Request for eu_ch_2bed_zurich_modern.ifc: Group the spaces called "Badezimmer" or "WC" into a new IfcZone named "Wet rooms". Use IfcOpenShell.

First a look at what the model holds.

```python
import ifcopenshell

model = ifcopenshell.open("eu_ch_2bed_zurich_modern.ifc")
print(model.schema)
seen = {}
for space in model.by_type("IfcSpace"):
    seen[space.LongName] = seen.get(space.LongName, 0) + 1
for name, count in sorted(seen.items(), key=str):
    print(count, "x", name)
print("zones:", [z.Name for z in model.by_type("IfcZone")][:20])
```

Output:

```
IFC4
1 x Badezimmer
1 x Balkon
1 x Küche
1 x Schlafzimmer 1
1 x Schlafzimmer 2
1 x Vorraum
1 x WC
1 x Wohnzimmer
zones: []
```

```python
import ifcopenshell
import ifcopenshell.api.group
import ifcopenshell.api.root

model = ifcopenshell.open("eu_ch_2bed_zurich_modern.ifc")

names = {"Badezimmer", "WC"}
spaces = [s for s in model.by_type("IfcSpace") if s.LongName in names]

zone = ifcopenshell.api.root.create_entity(model, ifc_class="IfcZone", name="Wet rooms")
ifcopenshell.api.group.assign_group(model, products=spaces, group=zone)
print(len(spaces), "spaces in", zone.Name)

model.write("eu_ch_2bed_zurich_modern_updated.ifc")
```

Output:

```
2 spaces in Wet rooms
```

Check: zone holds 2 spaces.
